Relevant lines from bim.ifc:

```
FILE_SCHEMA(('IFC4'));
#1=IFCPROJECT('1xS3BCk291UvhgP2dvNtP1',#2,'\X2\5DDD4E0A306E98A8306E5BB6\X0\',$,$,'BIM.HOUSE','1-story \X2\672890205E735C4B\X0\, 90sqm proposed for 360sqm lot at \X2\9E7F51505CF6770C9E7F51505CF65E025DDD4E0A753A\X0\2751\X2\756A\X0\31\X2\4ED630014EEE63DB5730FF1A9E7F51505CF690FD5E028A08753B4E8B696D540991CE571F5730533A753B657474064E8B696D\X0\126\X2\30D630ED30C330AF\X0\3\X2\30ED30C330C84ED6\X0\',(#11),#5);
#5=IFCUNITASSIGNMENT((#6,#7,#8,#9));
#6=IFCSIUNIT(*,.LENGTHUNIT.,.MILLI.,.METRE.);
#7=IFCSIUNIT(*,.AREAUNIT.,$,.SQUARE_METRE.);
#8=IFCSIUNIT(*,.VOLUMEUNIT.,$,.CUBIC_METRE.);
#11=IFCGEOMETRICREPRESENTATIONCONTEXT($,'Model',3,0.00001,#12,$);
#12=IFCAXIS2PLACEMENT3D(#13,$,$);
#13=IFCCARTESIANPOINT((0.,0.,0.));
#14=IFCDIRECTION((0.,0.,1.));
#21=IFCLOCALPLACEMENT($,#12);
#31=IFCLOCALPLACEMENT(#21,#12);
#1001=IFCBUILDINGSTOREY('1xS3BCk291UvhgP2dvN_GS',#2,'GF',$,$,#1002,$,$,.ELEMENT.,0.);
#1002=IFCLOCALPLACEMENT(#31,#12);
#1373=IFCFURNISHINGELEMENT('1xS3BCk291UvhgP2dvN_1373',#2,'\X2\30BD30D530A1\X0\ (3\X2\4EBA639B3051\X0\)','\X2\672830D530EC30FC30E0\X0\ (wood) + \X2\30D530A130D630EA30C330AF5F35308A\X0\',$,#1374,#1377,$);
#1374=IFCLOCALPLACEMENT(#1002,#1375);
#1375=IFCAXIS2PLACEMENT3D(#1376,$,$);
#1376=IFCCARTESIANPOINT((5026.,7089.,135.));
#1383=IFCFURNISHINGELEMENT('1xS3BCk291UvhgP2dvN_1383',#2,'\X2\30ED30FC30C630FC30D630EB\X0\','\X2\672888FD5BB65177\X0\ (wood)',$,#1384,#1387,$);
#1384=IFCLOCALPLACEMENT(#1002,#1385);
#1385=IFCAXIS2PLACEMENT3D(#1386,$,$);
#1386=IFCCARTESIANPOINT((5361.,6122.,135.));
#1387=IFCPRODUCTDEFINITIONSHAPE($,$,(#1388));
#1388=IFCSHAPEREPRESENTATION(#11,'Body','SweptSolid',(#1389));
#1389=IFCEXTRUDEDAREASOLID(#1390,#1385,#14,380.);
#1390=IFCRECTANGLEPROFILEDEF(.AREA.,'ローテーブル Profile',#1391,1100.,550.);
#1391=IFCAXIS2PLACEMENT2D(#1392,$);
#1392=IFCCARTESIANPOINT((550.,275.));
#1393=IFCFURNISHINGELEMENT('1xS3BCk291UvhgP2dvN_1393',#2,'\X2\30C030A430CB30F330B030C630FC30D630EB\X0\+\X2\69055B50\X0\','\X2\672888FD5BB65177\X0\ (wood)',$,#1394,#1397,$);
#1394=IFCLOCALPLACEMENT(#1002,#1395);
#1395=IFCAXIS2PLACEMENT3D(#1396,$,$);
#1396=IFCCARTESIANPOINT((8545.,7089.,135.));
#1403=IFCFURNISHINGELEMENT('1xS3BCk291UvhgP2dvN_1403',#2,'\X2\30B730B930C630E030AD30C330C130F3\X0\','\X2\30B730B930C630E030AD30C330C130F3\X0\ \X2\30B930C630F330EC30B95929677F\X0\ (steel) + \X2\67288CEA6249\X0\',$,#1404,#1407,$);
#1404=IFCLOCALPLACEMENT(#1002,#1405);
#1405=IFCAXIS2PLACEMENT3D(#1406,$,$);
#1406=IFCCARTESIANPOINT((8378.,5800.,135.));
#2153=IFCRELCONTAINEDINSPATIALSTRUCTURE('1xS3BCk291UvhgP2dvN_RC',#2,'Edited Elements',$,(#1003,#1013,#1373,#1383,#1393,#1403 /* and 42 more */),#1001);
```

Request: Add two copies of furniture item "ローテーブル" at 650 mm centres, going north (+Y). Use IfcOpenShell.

```python
import numpy as np
import ifcopenshell
import ifcopenshell.api.geometry
import ifcopenshell.api.root
import ifcopenshell.util.element
import ifcopenshell.util.placement
import ifcopenshell.util.unit

model = ifcopenshell.open("bim.ifc")
unit_scale = ifcopenshell.util.unit.calculate_unit_scale(model)


def reuse_history(source, copy):
    """copy_class also copies each property set's owner history, people and application; keep the originals."""
    for rel in copy.IsDefinedBy:
        if rel.is_a("IfcRelDefinesByProperties") and (history := rel.RelatingPropertyDefinition.OwnerHistory):
            rel.RelatingPropertyDefinition.OwnerHistory = source.OwnerHistory
            ifcopenshell.util.element.remove_deep2(model, history)


source = model.by_guid("1xS3BCk291UvhgP2dvN_1383")
base = ifcopenshell.util.placement.get_local_placement(source.ObjectPlacement)
step = np.array([0.0, 1.0, 0.0]) * 0.65 / unit_scale

for i in range(1, 3):
    copy = ifcopenshell.api.root.copy_class(model, product=source)
    copy.Representation = ifcopenshell.util.element.copy_deep(
        model, source.Representation, exclude=["IfcGeometricRepresentationContext", "IfcRepresentationMap"]
    )
    reuse_history(source, copy)
    matrix = base.copy()
    matrix[:3, 3] += i * step
    print("added at", matrix[:3, 3].round(3) + 0.0)
    ifcopenshell.api.geometry.edit_object_placement(model, product=copy, matrix=matrix, is_si=False)

model.write("bim_edited.ifc")
```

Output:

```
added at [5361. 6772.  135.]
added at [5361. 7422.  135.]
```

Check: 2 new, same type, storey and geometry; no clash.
